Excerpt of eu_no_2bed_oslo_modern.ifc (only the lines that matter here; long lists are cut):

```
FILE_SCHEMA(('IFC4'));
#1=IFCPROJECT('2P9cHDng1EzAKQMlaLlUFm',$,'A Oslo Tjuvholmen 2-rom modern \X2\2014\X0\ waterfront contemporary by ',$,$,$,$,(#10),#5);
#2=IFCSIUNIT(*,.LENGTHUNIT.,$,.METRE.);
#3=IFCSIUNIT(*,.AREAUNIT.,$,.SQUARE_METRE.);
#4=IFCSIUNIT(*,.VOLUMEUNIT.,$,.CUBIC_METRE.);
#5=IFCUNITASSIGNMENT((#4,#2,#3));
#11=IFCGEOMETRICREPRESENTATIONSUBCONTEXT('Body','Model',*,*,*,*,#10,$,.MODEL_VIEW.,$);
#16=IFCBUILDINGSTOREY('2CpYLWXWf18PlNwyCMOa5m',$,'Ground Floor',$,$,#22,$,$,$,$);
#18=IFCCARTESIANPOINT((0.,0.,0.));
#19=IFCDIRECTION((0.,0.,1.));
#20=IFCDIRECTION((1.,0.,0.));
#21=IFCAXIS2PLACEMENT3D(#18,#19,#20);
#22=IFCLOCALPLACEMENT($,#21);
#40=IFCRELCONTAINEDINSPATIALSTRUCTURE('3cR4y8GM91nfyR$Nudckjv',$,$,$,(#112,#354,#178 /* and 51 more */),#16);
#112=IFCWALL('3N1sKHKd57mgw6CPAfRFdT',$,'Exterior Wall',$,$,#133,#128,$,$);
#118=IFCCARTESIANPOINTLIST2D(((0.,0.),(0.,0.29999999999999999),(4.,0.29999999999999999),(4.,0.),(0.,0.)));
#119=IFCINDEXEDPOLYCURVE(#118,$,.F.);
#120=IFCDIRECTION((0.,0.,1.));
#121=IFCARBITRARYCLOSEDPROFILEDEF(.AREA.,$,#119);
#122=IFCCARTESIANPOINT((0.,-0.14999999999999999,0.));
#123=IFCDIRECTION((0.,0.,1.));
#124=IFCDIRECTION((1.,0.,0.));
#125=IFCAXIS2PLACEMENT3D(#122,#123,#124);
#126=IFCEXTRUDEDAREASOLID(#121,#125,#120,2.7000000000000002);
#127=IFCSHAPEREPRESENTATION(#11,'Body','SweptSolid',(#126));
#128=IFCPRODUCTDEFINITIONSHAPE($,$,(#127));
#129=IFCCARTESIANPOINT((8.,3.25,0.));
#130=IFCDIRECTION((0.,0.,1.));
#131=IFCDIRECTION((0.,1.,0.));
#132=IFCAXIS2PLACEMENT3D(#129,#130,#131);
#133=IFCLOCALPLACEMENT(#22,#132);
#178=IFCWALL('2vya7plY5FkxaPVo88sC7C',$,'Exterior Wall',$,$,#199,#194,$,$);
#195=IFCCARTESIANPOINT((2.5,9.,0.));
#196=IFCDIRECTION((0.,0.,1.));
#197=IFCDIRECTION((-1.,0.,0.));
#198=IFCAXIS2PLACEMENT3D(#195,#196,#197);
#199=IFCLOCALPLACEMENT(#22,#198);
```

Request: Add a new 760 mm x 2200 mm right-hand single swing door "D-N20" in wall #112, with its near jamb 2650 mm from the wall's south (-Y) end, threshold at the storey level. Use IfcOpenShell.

```python
import numpy as np
import ifcopenshell
import ifcopenshell.api.feature
import ifcopenshell.api.geometry
import ifcopenshell.api.root
import ifcopenshell.api.spatial
import ifcopenshell.geom
import ifcopenshell.util.element
import ifcopenshell.util.placement
import ifcopenshell.util.representation
import ifcopenshell.util.shape
import ifcopenshell.util.unit

model = ifcopenshell.open("eu_no_2bed_oslo_modern.ifc")
unit_scale = ifcopenshell.util.unit.calculate_unit_scale(model)
settings = ifcopenshell.geom.settings()


def volume(element):
    """Net volume in cubic metres, openings subtracted."""
    shape = ifcopenshell.geom.create_shape(settings, element)
    return ifcopenshell.util.shape.get_volume(shape.geometry)


wall = model.by_id(112)
storey = ifcopenshell.util.element.get_container(wall, ifc_class="IfcBuildingStorey")
context = ifcopenshell.util.representation.get_context(model, "Model", "Body", "MODEL_VIEW")
before = volume(wall)

width, height, from_end, sill = 0.76, 2.2, 2.65, 0.0  # metres

# The wall runs along its own X axis, and the end named is its -X end.
wall_shape = ifcopenshell.geom.create_shape(settings, wall)
x, y, z = ifcopenshell.util.shape.get_vertices(wall_shape.geometry).T
start = x.min() + from_end
face, thickness = float(y.min()), float(y.max() - y.min())
wall_matrix = ifcopenshell.util.placement.get_local_placement(wall.ObjectPlacement)
level = ifcopenshell.util.placement.get_local_placement(storey.ObjectPlacement)[2, 3]


def in_wall(x, y):
    """Placement at x, y metres in the wall's axes, at sill height."""
    matrix = wall_matrix.copy()
    matrix[:, 3] = wall_matrix @ np.array([x / unit_scale, y / unit_scale, 0.0, 1.0])
    matrix[2, 3] = level + sill / unit_scale
    return matrix


# Opening: a box that overshoots both wall faces by 50 mm.
opening = ifcopenshell.api.root.create_entity(model, ifc_class="IfcOpeningElement", predefined_type="OPENING")
box = ifcopenshell.api.geometry.add_wall_representation(
    model, context=context, length=width, height=height, thickness=thickness + 0.1
)
ifcopenshell.api.geometry.assign_representation(model, product=opening, representation=box)
ifcopenshell.api.geometry.edit_object_placement(model, product=opening, matrix=in_wall(start, face - 0.05), is_si=False)
ifcopenshell.api.feature.add_feature(model, feature=opening, element=wall)

door = ifcopenshell.api.root.create_entity(model, ifc_class="IfcDoor", name="D-N20", predefined_type="DOOR")
door.OverallWidth, door.OverallHeight = width / unit_scale, height / unit_scale
door.OperationType = "SINGLE_SWING_RIGHT"
body = ifcopenshell.api.geometry.add_door_representation(
    model,
    context=context,
    overall_width=door.OverallWidth,
    overall_height=door.OverallHeight,
    operation_type="SINGLE_SWING_RIGHT",
    lining_properties={"LiningDepth": thickness / unit_scale, "ThresholdDepth": thickness / unit_scale},
)
ifcopenshell.api.geometry.assign_representation(model, product=door, representation=body)
ifcopenshell.api.spatial.assign_container(model, products=[door], relating_structure=storey)
ifcopenshell.api.feature.add_filling(model, opening=opening, element=door)

# The lining spans the wall, so the door starts at the wall face.
ifcopenshell.api.geometry.edit_object_placement(model, product=door, matrix=in_wall(start, face), is_si=False)

after = volume(wall)

print(f"wall volume {before:.3f} -> {after:.3f} m3")

model.write("eu_no_2bed_oslo_modern-out.ifc")
```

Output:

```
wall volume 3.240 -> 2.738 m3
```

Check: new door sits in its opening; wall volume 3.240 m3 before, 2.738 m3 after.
